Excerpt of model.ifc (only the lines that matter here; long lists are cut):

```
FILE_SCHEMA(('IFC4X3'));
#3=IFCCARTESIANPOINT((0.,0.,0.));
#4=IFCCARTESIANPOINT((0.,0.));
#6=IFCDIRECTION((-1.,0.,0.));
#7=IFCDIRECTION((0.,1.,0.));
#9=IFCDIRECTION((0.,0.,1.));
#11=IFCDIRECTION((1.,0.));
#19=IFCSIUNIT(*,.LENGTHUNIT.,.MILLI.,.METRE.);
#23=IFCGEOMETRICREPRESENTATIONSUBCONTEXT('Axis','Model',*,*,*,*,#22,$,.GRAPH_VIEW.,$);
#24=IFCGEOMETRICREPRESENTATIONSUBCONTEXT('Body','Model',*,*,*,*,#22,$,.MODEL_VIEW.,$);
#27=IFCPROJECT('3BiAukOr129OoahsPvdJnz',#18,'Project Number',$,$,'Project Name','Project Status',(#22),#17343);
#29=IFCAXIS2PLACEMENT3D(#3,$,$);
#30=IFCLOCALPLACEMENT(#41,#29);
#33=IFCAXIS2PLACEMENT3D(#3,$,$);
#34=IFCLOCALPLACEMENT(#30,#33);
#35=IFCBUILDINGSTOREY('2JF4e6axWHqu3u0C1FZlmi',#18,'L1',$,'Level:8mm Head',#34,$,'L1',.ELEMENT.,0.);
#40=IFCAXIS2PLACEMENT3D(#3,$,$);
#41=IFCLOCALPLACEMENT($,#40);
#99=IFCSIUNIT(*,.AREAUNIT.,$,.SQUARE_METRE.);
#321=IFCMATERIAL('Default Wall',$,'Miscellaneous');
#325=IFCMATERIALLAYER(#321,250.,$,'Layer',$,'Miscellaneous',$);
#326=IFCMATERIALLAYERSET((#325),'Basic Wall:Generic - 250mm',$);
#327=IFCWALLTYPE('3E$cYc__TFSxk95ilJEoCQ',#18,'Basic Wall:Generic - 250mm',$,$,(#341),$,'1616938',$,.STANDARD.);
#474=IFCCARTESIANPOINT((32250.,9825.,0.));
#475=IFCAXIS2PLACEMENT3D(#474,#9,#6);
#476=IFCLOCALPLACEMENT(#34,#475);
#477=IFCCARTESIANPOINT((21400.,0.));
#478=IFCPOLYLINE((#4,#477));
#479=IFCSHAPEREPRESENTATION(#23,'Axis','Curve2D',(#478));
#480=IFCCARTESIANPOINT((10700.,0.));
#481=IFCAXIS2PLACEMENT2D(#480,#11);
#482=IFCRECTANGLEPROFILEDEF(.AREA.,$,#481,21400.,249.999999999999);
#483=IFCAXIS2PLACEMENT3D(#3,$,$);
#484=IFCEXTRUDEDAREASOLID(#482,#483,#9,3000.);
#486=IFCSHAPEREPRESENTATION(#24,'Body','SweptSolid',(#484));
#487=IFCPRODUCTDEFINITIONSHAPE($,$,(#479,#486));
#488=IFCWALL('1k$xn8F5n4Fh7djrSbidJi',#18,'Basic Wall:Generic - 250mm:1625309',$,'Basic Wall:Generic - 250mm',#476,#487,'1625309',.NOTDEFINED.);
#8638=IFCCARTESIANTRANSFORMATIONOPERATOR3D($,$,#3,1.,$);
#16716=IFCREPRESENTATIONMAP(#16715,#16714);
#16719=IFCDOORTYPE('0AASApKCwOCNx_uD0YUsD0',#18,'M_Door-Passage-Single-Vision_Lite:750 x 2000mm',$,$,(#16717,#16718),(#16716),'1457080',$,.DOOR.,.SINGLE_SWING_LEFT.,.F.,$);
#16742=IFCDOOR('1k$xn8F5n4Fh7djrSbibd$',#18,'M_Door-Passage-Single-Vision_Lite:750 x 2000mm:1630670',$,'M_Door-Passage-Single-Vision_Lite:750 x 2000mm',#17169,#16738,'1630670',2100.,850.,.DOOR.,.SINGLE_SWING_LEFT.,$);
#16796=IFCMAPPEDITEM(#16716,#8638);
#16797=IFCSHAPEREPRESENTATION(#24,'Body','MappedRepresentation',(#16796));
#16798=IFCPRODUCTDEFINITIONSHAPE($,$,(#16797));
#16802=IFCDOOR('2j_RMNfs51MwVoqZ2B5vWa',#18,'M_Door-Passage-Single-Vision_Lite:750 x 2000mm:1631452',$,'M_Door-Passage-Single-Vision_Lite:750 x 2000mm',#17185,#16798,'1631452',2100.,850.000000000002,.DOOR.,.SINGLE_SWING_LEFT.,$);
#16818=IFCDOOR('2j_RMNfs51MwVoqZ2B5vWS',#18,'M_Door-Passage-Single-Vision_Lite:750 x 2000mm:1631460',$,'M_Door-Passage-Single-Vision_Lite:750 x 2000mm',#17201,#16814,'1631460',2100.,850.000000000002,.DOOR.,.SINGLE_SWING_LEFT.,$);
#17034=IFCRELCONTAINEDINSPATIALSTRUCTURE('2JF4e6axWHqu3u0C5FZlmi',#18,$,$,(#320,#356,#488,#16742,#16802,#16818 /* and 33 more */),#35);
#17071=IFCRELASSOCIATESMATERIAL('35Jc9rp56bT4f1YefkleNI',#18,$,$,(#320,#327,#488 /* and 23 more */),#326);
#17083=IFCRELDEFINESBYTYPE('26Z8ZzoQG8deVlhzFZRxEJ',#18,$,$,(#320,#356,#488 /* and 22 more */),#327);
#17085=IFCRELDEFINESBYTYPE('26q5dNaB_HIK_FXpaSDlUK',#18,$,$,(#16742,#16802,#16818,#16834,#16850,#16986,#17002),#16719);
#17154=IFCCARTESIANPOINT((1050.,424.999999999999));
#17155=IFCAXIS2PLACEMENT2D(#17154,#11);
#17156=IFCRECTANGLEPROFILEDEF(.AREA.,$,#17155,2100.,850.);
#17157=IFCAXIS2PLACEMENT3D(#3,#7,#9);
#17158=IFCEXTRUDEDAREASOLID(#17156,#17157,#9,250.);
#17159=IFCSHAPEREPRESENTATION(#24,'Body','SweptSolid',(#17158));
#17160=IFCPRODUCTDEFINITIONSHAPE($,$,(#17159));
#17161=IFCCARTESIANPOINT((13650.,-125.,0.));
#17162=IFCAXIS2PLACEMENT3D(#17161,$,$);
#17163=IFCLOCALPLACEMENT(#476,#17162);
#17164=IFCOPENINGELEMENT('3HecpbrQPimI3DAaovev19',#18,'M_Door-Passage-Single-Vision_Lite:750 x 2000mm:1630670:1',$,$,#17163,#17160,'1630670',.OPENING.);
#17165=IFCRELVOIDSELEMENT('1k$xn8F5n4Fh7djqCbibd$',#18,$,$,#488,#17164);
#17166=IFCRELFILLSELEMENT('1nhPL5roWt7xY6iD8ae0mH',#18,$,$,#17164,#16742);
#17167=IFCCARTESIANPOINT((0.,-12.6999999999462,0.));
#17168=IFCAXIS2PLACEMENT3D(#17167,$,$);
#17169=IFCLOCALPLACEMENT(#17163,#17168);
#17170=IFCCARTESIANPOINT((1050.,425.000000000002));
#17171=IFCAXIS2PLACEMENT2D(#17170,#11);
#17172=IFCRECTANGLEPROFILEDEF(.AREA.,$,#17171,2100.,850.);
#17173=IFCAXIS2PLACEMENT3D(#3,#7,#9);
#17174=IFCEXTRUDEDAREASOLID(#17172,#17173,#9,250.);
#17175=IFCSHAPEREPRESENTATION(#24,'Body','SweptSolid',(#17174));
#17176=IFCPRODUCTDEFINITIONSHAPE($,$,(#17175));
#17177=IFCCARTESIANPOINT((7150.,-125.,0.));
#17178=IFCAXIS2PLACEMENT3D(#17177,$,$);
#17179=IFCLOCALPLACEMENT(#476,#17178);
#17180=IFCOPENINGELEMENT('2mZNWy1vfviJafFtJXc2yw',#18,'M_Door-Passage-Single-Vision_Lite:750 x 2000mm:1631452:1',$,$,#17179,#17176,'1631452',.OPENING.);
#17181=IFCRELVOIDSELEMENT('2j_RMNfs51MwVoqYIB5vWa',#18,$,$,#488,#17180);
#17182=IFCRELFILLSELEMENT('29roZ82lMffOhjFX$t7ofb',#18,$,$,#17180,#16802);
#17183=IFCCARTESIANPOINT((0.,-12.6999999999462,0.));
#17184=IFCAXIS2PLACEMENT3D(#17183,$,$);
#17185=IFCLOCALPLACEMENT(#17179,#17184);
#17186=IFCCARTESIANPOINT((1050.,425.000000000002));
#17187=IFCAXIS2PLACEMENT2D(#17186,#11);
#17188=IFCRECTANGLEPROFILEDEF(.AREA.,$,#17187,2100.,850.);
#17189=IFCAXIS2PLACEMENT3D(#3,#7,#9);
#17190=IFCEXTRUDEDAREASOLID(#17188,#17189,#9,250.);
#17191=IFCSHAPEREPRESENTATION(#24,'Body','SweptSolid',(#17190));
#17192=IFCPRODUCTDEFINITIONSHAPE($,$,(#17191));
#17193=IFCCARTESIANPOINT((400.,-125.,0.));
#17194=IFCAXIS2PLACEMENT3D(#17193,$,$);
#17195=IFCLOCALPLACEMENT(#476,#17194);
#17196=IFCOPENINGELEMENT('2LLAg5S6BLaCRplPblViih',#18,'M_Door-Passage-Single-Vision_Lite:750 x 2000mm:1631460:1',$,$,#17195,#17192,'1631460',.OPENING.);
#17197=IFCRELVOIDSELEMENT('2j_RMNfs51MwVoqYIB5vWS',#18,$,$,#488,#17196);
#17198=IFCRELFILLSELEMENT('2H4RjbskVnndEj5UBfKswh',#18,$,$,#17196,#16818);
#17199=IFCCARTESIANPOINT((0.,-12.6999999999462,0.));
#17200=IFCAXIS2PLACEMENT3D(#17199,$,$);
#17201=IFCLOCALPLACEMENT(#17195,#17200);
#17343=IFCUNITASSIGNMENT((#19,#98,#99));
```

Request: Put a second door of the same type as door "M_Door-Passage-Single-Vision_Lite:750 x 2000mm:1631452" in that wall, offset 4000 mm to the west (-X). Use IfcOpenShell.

```python
import ifcopenshell
import ifcopenshell.api.feature
import ifcopenshell.api.geometry
import ifcopenshell.api.root
import ifcopenshell.geom
import ifcopenshell.util.element
import ifcopenshell.util.placement
import ifcopenshell.util.shape

model = ifcopenshell.open("model.ifc")
settings = ifcopenshell.geom.settings()


def volume(element):
    """Net volume in cubic metres, openings subtracted."""
    shape = ifcopenshell.geom.create_shape(settings, element)
    return ifcopenshell.util.shape.get_volume(shape.geometry)


def reuse_history(source, copy):
    """copy_class also copies each property set's owner history, people and application; keep the originals."""
    for rel in copy.IsDefinedBy:
        if rel.is_a("IfcRelDefinesByProperties") and (history := rel.RelatingPropertyDefinition.OwnerHistory):
            rel.RelatingPropertyDefinition.OwnerHistory = source.OwnerHistory
            ifcopenshell.util.element.remove_deep2(model, history)


door = model.by_id(16802)
opening = door.FillsVoids[0].RelatingOpeningElement
wall = opening.VoidsElements[0].RelatingBuildingElement
before = volume(wall)
shift = ifcopenshell.util.placement.get_local_placement(wall.ObjectPlacement)[:3, 0] * 4000.0

# copy_class copies the void relationship, type, container and properties, but no geometry.
new_opening = ifcopenshell.api.root.copy_class(model, product=opening)
new_opening.Representation = ifcopenshell.util.element.copy_deep(
    model, opening.Representation, exclude=["IfcGeometricRepresentationContext", "IfcRepresentationMap"]
)
new_opening.Name = "M_Door-Passage-Single-Vision_Lite:750 x 2000mm"
new_opening.Tag = None
new_door = ifcopenshell.api.root.copy_class(model, product=door)
new_door.Representation = ifcopenshell.util.element.copy_deep(
    model, door.Representation, exclude=["IfcGeometricRepresentationContext", "IfcRepresentationMap"]
)
new_door.Name = "M_Door-Passage-Single-Vision_Lite:750 x 2000mm"
new_door.Tag = None
reuse_history(door, new_door)
ifcopenshell.api.feature.add_filling(model, opening=new_opening, element=new_door)

for old, new in ((opening, new_opening), (door, new_door)):
    matrix = ifcopenshell.util.placement.get_local_placement(old.ObjectPlacement)
    matrix[:3, 3] += shift
    ifcopenshell.api.geometry.edit_object_placement(model, product=new, matrix=matrix, is_si=False)

after = volume(wall)

print(f"wall volume {before:.3f} -> {after:.3f} m3")

model.write("model_updated.ifc")
```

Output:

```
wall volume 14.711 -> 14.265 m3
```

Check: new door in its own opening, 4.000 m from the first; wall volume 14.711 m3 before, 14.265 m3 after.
